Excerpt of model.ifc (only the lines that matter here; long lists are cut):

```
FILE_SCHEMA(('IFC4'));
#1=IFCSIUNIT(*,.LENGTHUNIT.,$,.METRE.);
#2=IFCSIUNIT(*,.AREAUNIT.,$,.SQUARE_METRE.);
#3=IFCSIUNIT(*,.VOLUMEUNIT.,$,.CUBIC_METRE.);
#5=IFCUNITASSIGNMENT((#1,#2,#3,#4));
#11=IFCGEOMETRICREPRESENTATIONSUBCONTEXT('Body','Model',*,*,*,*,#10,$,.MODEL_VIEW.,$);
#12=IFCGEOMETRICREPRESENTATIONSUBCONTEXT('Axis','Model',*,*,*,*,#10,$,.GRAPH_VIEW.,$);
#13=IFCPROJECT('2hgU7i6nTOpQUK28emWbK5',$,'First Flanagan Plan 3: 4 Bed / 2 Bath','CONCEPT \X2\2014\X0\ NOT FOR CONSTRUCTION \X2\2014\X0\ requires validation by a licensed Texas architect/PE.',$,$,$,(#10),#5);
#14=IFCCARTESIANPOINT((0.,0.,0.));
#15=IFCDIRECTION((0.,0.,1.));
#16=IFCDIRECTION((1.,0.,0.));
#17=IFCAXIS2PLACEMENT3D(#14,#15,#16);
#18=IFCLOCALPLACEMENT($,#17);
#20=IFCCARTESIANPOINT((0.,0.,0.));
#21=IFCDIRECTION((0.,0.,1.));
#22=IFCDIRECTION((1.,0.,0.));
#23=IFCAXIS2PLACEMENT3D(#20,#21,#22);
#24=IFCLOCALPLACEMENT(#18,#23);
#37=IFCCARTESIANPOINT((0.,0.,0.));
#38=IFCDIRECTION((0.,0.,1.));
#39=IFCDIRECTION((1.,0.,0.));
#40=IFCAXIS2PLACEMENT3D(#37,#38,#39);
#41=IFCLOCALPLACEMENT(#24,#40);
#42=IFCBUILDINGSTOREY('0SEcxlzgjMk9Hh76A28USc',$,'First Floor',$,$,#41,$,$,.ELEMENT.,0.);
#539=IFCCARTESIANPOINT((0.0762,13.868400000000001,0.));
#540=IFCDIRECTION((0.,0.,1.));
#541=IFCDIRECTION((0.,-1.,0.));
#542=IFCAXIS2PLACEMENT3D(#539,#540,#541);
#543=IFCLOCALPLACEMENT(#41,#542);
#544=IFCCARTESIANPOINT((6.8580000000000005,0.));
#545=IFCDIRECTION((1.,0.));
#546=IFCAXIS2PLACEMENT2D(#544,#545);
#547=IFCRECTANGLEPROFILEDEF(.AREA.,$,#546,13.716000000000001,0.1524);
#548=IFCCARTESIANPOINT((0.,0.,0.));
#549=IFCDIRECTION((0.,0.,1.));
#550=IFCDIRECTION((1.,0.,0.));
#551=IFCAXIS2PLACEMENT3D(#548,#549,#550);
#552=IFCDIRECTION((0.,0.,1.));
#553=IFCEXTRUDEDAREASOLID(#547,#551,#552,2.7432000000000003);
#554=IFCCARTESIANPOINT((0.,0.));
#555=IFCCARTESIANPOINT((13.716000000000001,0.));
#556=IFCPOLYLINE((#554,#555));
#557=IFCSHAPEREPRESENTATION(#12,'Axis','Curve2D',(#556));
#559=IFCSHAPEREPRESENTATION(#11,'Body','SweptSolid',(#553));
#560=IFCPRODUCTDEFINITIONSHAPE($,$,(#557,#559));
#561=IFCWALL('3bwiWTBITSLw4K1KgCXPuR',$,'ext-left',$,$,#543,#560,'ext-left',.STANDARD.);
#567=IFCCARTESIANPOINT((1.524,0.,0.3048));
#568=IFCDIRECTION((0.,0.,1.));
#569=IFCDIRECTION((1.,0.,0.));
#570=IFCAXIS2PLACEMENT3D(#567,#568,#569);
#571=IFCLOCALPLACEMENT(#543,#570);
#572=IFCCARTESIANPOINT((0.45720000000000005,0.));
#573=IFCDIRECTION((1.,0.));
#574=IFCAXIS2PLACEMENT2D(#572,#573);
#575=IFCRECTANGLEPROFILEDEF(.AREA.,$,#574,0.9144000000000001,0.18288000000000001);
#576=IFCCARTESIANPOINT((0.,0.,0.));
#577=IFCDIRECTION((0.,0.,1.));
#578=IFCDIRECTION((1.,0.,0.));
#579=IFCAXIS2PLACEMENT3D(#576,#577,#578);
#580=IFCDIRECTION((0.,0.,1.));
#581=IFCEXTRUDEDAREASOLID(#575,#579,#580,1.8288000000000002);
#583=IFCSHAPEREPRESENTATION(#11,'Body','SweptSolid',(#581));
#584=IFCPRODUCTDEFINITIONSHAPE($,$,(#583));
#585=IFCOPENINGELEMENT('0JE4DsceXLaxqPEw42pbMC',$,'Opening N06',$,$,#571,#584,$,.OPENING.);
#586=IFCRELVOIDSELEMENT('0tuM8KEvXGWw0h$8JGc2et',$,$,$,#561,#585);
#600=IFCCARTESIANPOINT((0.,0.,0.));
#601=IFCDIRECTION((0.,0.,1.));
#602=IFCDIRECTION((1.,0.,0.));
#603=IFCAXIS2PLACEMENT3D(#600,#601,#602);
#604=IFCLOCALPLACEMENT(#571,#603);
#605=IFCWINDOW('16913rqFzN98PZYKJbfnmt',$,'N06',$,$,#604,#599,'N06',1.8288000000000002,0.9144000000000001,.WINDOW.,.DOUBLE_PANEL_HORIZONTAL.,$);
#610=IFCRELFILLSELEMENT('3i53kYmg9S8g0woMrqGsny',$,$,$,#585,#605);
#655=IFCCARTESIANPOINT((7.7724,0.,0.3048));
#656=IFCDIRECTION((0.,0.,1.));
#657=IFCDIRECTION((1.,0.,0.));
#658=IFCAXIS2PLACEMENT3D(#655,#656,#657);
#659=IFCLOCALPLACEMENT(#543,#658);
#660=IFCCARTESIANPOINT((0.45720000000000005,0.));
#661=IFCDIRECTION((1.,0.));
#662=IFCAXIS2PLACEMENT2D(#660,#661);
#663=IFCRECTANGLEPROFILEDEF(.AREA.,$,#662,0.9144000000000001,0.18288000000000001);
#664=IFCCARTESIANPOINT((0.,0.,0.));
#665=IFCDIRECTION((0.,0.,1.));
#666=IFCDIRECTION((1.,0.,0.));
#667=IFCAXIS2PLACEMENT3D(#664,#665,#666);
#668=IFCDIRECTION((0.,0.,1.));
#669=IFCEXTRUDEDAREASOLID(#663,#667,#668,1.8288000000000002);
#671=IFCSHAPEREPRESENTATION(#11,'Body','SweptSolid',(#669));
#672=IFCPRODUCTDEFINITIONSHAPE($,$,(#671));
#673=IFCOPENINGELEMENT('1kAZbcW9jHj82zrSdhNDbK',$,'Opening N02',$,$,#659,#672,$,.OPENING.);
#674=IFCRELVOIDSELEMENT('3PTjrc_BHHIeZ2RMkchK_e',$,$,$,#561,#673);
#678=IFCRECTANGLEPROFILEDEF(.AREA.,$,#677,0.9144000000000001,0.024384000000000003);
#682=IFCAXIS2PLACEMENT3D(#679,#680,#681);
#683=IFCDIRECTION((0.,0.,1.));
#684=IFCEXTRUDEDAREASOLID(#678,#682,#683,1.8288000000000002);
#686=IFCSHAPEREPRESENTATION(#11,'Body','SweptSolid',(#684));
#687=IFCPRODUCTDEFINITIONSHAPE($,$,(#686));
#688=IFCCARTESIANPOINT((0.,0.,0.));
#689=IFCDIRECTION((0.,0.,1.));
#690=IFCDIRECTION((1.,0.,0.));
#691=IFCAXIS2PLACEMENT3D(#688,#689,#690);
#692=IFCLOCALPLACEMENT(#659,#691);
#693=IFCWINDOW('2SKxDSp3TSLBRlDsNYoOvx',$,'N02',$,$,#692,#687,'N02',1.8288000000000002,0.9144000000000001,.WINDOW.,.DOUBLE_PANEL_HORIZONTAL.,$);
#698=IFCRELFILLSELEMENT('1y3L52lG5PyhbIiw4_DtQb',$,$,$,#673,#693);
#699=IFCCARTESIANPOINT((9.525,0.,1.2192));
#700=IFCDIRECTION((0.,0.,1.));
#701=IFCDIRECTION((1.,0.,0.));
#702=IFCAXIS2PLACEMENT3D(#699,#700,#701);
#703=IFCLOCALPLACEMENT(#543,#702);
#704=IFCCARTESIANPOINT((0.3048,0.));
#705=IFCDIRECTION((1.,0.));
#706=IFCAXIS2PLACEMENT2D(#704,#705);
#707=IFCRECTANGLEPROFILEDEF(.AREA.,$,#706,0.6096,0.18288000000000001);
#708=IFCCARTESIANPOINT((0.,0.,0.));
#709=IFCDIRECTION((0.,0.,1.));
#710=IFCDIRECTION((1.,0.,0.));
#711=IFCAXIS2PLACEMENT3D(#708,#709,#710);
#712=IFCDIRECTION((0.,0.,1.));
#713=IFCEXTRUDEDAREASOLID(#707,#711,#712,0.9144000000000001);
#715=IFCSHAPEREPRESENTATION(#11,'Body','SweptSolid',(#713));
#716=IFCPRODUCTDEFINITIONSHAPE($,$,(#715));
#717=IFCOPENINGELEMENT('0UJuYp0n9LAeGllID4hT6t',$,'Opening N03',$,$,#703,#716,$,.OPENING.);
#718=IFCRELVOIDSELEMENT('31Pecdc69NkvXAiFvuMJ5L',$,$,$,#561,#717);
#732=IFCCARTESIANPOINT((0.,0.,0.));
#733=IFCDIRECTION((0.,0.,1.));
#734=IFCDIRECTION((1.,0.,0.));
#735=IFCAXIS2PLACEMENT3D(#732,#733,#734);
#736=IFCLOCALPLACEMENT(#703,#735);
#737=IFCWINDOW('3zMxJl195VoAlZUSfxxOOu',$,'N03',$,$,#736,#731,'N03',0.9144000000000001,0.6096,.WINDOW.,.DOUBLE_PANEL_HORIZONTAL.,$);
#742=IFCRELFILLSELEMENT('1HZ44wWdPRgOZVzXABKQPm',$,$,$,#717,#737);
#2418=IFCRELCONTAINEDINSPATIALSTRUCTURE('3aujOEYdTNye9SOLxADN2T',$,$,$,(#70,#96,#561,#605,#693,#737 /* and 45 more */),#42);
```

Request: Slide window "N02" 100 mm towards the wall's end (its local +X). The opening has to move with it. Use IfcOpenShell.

```python
import ifcopenshell
import ifcopenshell.api.geometry
import ifcopenshell.util.placement
import ifcopenshell.util.unit

model = ifcopenshell.open("model.ifc")
unit_scale = ifcopenshell.util.unit.calculate_unit_scale(model)

window = model.by_guid("2SKxDSp3TSLBRlDsNYoOvx")
opening = window.FillsVoids[0].RelatingOpeningElement
wall = opening.VoidsElements[0].RelatingBuildingElement

wall_matrix = ifcopenshell.util.placement.get_local_placement(wall.ObjectPlacement)
shift = wall_matrix[:3, 0] * 0.1 / unit_scale
before = ifcopenshell.util.placement.get_local_placement(window.ObjectPlacement)[:3, 3].copy()

# The window is placed relative to its opening, so it follows when the opening moves.
matrix = ifcopenshell.util.placement.get_local_placement(opening.ObjectPlacement)
matrix[:3, 3] += shift
ifcopenshell.api.geometry.edit_object_placement(
    model, product=opening, matrix=matrix, is_si=False, should_transform_children=True
)

after = ifcopenshell.util.placement.get_local_placement(window.ObjectPlacement)[:3, 3]
print("window moved by", (after - before).round(3) + 0.0)

model.write("model_v2.ifc")
```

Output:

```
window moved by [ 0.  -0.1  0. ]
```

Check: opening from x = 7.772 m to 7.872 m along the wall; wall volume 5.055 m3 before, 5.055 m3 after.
